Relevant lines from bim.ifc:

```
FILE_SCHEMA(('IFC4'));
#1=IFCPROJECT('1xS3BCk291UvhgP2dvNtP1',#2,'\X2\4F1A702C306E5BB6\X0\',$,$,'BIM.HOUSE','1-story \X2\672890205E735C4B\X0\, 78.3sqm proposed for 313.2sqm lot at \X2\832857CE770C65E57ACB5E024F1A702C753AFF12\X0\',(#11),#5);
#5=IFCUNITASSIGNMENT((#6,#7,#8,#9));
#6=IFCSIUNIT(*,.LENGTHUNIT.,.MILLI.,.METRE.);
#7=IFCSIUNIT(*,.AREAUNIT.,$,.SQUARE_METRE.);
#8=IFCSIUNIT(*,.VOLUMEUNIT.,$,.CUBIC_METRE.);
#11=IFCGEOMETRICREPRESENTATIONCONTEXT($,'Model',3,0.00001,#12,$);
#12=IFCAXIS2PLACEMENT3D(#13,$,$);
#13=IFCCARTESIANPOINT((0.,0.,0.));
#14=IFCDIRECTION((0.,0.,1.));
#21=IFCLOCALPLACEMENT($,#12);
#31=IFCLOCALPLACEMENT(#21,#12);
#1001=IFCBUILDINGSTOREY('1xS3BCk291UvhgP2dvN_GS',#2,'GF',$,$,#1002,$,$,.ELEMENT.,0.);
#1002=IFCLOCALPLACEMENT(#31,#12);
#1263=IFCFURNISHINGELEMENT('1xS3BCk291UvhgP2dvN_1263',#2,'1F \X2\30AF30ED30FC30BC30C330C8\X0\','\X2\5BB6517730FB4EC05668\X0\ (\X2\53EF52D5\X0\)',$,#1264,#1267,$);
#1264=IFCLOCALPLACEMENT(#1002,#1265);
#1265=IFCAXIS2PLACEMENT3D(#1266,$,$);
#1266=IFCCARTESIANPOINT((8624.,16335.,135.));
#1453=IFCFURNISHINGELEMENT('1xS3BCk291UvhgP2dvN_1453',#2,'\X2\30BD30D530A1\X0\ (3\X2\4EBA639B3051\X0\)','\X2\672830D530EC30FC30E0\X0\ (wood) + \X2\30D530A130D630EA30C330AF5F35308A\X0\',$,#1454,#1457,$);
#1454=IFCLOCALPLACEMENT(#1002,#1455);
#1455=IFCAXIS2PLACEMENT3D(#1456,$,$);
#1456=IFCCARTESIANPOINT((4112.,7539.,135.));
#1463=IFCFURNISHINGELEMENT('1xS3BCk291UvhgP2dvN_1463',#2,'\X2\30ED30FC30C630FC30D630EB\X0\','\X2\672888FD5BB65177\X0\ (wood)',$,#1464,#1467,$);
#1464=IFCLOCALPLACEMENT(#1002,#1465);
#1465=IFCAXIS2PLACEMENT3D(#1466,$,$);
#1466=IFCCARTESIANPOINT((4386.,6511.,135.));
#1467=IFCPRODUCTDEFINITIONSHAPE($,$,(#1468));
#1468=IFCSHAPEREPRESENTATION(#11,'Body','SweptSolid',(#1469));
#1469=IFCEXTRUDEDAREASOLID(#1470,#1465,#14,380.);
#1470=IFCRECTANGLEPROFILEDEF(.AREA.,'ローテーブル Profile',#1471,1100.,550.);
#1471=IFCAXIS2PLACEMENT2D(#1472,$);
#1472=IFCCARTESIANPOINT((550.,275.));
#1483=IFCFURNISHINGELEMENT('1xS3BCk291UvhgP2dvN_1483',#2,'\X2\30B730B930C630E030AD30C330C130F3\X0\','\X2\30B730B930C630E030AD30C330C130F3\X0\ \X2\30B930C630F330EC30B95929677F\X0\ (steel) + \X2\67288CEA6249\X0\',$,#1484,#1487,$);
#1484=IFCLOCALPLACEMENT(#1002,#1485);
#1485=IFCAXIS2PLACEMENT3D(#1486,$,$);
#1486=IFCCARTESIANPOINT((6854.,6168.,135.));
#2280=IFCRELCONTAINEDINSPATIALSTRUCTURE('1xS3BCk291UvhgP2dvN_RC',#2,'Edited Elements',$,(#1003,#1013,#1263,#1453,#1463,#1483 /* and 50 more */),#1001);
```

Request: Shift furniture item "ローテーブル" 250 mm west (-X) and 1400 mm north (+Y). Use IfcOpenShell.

```python
import ifcopenshell
import ifcopenshell.api.geometry
import ifcopenshell.util.placement
import ifcopenshell.util.unit

model = ifcopenshell.open("bim.ifc")
unit_scale = ifcopenshell.util.unit.calculate_unit_scale(model)

item = model.by_guid("1xS3BCk291UvhgP2dvN_1463")
matrix = ifcopenshell.util.placement.get_local_placement(item.ObjectPlacement)
matrix[0, 3] -= 0.25 / unit_scale
matrix[1, 3] += 1.4 / unit_scale
ifcopenshell.api.geometry.edit_object_placement(model, product=item, matrix=matrix, is_si=False)

print(ifcopenshell.util.placement.get_local_placement(item.ObjectPlacement).round(3) + 0.0)

model.write("bim_rev.ifc")
```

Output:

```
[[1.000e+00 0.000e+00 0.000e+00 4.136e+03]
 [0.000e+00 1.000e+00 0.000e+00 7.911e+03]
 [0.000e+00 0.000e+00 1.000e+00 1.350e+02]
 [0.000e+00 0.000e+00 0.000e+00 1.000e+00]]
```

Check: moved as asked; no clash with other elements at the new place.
